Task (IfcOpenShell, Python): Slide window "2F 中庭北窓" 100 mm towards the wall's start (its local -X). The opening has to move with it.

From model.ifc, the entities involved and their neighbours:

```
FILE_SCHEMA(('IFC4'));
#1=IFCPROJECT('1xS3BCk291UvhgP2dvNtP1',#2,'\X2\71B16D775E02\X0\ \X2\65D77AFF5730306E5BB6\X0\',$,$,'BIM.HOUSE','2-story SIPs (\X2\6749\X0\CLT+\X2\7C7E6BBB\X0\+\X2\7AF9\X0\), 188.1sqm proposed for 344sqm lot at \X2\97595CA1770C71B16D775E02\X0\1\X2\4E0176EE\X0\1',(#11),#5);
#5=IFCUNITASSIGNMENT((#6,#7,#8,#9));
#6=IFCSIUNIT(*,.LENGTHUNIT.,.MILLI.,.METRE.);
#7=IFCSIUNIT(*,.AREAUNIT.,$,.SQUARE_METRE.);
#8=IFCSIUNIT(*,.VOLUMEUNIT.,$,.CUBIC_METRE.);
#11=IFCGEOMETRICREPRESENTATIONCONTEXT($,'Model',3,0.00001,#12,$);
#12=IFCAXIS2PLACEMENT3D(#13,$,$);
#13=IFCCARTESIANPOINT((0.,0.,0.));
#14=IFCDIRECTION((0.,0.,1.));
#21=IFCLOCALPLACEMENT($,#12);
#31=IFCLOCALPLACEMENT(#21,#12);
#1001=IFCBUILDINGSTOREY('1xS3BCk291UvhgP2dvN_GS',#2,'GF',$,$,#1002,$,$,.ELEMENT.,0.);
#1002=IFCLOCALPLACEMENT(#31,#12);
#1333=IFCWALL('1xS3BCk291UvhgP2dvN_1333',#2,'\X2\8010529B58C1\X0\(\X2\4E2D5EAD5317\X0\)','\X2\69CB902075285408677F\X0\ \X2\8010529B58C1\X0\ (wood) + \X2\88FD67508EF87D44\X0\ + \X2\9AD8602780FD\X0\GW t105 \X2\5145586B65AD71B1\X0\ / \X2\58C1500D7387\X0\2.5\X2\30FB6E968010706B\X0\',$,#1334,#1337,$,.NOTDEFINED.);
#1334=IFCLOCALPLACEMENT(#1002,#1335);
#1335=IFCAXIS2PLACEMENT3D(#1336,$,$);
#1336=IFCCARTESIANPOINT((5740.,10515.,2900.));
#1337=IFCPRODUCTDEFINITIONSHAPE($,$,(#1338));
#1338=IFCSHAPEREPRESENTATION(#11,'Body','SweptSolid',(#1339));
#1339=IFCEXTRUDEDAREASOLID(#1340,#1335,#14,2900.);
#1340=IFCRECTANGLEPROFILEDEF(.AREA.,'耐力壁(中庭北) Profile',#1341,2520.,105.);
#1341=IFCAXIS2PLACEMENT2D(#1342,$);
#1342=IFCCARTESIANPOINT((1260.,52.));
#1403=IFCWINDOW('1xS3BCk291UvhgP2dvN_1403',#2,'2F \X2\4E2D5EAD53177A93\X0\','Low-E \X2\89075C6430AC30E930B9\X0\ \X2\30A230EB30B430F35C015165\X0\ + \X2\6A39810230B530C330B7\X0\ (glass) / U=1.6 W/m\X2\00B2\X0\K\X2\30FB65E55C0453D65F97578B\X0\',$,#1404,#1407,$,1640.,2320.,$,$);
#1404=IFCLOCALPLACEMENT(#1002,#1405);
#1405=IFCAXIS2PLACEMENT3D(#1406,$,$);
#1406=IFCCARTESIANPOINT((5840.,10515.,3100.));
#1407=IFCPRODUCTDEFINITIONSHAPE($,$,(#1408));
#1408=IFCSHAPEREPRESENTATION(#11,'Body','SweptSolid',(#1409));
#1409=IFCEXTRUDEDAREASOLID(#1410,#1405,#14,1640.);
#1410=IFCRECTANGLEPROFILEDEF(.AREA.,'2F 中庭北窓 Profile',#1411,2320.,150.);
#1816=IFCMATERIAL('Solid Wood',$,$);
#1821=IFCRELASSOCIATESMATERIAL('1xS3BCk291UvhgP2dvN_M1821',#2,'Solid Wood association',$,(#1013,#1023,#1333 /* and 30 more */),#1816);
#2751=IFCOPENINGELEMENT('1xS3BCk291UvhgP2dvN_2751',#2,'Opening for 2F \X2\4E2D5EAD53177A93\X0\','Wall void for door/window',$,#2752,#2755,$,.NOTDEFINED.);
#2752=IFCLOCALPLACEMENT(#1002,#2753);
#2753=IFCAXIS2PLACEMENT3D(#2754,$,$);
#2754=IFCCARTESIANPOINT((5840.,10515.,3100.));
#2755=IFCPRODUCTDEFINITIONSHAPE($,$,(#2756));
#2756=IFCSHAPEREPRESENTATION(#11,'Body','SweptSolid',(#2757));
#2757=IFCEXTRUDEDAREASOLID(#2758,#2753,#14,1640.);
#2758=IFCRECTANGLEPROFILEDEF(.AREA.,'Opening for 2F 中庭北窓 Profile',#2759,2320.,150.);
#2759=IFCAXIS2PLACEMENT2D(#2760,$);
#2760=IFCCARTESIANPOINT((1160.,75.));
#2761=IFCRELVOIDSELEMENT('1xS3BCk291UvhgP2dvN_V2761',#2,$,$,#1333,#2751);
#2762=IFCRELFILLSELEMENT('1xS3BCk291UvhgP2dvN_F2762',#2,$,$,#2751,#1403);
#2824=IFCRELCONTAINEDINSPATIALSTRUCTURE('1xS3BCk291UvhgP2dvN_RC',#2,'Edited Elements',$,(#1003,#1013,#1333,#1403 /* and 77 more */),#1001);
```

```python
import ifcopenshell
import ifcopenshell.api.geometry
import ifcopenshell.util.placement
import ifcopenshell.util.unit

model = ifcopenshell.open("model.ifc")
unit_scale = ifcopenshell.util.unit.calculate_unit_scale(model)

window = model.by_guid("1xS3BCk291UvhgP2dvN_1403")
opening = window.FillsVoids[0].RelatingOpeningElement
wall = opening.VoidsElements[0].RelatingBuildingElement

wall_matrix = ifcopenshell.util.placement.get_local_placement(wall.ObjectPlacement)
shift = wall_matrix[:3, 0] * -0.1 / unit_scale
before = ifcopenshell.util.placement.get_local_placement(window.ObjectPlacement)[:3, 3].copy()

# The window is not placed relative to its opening, so move both.
for product in (opening, window):
    matrix = ifcopenshell.util.placement.get_local_placement(product.ObjectPlacement)
    matrix[:3, 3] += shift
    ifcopenshell.api.geometry.edit_object_placement(model, product=product, matrix=matrix, is_si=False)

after = ifcopenshell.util.placement.get_local_placement(window.ObjectPlacement)[:3, 3]
print("window moved by", (after - before).round(3) + 0.0)

model.write("model_updated.ifc")
```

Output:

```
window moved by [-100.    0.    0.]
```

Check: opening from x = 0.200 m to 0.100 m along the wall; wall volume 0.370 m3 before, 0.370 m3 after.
